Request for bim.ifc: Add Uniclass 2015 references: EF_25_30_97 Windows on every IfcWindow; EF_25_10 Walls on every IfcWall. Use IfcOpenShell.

First a look at what the model holds.

```python
import ifcopenshell

model = ifcopenshell.open("bim.ifc")
print(model.schema)
print("classifications:", [c.Name for c in model.by_type("IfcClassification")])
for ifc_class in ("IfcDoor", "IfcRoof", "IfcStair", "IfcWall", "IfcWindow"):
    print(ifc_class, len(model.by_type(ifc_class)))
```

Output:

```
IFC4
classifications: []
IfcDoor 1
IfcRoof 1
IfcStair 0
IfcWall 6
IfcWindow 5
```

```python
import ifcopenshell
import ifcopenshell.api.classification

model = ifcopenshell.open("bim.ifc")

system = ifcopenshell.api.classification.add_classification(model, classification="Uniclass 2015")

codes = {
    "IfcWindow": ("EF_25_30_97", "Windows"),
    "IfcWall": ("EF_25_10", "Walls"),
}
for ifc_class, (code, name) in codes.items():
    products = model.by_type(ifc_class)
    ifcopenshell.api.classification.add_reference(
        model, products=products, classification=system, identification=code, name=name
    )
    print(code, len(products))

model.write("bim_v2.ifc")
```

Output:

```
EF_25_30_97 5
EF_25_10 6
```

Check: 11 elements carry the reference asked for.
